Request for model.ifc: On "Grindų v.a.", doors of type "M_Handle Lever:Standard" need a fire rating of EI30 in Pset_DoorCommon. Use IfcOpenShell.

First a look at what the model holds.

```python
import ifcopenshell
import ifcopenshell.util.element

model = ifcopenshell.open("model.ifc")
print(model.schema)
storey = next(s for s in model.by_type("IfcBuildingStorey") if s.Name == "Grindų v.a.")
doors = [e for e in ifcopenshell.util.element.get_decomposition(storey) if e.is_a("IfcDoor")]
seen = {}
for e in doors:
    element_type = ifcopenshell.util.element.get_type(e)
    key = (element_type.Name if element_type != e and element_type else None, ifcopenshell.util.element.get_pset(e, "Pset_DoorCommon", "FireRating"))
    seen[key] = seen.get(key, 0) + 1
for (name, value), count in sorted(seen.items(), key=str):
    print(count, "x", name, "|", value)
```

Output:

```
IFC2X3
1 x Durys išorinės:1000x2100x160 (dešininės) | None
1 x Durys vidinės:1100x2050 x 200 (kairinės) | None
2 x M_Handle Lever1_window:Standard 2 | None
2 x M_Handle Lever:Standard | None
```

```python
import ifcopenshell
import ifcopenshell.api.pset
import ifcopenshell.util.element

model = ifcopenshell.open("model.ifc")

storey = next(s for s in model.by_type("IfcBuildingStorey") if s.Name == "Grindų v.a.")
doors = [e for e in ifcopenshell.util.element.get_decomposition(storey) if e.is_a("IfcDoor")]

count = 0
for e in doors:
    element_type = ifcopenshell.util.element.get_type(e)
    if element_type in (None, e) or element_type.Name != "M_Handle Lever:Standard":
        continue
    # add_pset returns the element's existing set when there is one.
    pset = ifcopenshell.api.pset.add_pset(model, product=e, name="Pset_DoorCommon")
    ifcopenshell.api.pset.edit_pset(model, pset=pset, properties={"FireRating": "EI30"})
    count += 1

print(count, "doors updated")

model.write("model_rev.ifc")
```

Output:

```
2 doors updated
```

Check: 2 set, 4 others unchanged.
